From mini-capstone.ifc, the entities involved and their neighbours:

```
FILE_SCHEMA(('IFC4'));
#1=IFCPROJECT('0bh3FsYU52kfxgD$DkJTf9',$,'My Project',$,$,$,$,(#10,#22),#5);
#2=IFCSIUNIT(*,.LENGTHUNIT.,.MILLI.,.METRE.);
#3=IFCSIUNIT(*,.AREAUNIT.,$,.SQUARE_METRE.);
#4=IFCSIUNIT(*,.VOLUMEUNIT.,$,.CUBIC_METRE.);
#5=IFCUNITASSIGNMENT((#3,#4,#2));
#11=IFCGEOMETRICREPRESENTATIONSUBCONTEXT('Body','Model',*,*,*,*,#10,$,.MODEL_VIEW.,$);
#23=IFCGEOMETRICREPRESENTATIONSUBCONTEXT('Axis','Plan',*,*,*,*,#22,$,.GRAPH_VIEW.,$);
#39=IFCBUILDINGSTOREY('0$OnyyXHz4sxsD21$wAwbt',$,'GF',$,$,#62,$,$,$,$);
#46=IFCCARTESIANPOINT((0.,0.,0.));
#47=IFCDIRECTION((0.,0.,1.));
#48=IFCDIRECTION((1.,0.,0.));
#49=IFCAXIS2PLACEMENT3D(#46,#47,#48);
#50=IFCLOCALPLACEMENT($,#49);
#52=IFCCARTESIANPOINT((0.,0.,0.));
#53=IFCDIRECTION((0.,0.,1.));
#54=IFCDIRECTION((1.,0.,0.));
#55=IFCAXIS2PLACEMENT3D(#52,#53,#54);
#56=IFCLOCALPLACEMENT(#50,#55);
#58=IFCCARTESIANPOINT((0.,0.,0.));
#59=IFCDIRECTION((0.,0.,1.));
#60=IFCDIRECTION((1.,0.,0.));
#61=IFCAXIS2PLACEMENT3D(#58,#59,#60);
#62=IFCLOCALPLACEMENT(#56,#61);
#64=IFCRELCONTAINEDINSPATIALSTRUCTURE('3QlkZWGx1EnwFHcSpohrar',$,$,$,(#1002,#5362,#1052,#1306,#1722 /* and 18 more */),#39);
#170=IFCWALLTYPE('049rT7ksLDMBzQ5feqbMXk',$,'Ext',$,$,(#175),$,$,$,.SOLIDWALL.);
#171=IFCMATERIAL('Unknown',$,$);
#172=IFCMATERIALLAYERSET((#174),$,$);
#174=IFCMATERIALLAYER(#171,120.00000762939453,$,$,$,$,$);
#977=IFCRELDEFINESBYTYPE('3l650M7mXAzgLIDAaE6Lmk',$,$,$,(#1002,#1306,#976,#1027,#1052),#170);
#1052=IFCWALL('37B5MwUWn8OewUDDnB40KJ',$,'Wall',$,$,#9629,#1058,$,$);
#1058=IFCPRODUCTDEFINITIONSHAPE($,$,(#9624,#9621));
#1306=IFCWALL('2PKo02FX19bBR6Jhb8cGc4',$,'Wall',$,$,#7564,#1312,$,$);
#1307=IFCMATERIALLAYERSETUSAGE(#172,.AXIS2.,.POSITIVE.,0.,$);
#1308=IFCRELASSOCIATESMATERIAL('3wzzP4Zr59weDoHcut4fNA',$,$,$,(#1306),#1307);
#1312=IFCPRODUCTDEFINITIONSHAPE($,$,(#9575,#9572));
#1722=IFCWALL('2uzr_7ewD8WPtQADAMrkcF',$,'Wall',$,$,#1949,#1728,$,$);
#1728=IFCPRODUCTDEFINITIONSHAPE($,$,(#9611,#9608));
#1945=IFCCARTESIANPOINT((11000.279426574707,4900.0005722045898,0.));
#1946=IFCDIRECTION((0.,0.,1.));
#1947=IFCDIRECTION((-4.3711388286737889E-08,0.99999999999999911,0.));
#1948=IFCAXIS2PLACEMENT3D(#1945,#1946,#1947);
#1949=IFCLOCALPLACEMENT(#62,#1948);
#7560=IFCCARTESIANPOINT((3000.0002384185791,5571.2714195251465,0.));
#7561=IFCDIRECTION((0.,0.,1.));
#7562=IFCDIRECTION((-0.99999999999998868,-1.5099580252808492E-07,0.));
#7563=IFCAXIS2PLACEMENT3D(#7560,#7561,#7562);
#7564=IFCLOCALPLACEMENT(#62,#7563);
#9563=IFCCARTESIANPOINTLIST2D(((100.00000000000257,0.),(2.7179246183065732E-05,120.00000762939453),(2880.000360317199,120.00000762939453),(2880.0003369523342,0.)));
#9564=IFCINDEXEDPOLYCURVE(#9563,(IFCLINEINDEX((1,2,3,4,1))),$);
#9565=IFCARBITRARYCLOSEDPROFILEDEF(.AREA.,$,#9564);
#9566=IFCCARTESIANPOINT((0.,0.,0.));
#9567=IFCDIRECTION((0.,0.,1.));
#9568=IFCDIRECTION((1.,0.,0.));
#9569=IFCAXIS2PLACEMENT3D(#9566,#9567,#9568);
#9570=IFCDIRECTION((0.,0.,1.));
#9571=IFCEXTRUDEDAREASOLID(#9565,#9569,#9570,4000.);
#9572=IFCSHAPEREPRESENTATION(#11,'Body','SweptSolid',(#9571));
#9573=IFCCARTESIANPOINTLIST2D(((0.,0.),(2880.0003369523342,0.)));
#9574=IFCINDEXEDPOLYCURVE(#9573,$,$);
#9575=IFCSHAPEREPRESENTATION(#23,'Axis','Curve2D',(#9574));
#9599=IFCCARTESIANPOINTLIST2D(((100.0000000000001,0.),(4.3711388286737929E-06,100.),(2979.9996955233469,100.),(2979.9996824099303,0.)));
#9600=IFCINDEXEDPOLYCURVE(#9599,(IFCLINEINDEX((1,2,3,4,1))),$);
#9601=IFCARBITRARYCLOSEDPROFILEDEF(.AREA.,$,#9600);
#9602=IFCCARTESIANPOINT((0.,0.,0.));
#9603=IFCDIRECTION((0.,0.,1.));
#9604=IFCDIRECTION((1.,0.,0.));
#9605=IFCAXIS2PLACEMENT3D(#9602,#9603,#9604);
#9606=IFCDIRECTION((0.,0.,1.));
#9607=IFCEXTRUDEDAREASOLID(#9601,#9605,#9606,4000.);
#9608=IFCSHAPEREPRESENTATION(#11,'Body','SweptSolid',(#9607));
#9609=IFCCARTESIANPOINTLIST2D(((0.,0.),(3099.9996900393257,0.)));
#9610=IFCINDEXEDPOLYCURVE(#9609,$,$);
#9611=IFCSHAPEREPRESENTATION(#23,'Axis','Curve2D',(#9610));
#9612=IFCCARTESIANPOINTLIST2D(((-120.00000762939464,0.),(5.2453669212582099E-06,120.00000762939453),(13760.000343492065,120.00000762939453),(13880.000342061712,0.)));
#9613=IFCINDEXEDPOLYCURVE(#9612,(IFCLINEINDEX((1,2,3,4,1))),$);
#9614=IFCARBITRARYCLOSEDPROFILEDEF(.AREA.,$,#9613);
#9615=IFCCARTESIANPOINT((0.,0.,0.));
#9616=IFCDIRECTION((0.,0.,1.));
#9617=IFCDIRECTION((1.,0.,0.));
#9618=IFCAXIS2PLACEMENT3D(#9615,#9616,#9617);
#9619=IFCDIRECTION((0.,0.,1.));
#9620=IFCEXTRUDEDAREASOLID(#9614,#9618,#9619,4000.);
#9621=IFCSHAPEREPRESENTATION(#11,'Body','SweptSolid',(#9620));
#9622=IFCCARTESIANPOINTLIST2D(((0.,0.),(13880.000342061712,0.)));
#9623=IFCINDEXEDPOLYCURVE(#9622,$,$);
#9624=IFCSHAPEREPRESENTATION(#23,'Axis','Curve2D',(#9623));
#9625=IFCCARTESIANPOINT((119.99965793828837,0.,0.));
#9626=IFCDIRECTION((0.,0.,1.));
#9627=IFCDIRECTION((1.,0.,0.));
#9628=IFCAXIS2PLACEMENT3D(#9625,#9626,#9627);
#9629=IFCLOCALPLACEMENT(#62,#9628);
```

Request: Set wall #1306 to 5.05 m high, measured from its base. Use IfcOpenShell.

```python
import ifcopenshell
import ifcopenshell.geom
import ifcopenshell.util.representation
import ifcopenshell.util.shape
import ifcopenshell.util.unit

model = ifcopenshell.open("mini-capstone.ifc")
unit_scale = ifcopenshell.util.unit.calculate_unit_scale(model)
settings = ifcopenshell.geom.settings()


def volume(element):
    """Net volume in cubic metres, openings subtracted."""
    shape = ifcopenshell.geom.create_shape(settings, element)
    return ifcopenshell.util.shape.get_volume(shape.geometry)


wall = model.by_id(1306)
before = volume(wall)

body = ifcopenshell.util.representation.get_representation(wall, "Model", "Body")
solid = body.Items[0]
old_height = solid.Depth
solid.Depth = 5.05 / unit_scale
after = volume(wall)

print(f"height {old_height:g} -> {solid.Depth:g}, volume {before:.3f} -> {after:.3f} m3")

model.write("mini-capstone_edited.ifc")
```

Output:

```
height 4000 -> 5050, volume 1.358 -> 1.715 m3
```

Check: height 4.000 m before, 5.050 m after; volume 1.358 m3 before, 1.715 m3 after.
